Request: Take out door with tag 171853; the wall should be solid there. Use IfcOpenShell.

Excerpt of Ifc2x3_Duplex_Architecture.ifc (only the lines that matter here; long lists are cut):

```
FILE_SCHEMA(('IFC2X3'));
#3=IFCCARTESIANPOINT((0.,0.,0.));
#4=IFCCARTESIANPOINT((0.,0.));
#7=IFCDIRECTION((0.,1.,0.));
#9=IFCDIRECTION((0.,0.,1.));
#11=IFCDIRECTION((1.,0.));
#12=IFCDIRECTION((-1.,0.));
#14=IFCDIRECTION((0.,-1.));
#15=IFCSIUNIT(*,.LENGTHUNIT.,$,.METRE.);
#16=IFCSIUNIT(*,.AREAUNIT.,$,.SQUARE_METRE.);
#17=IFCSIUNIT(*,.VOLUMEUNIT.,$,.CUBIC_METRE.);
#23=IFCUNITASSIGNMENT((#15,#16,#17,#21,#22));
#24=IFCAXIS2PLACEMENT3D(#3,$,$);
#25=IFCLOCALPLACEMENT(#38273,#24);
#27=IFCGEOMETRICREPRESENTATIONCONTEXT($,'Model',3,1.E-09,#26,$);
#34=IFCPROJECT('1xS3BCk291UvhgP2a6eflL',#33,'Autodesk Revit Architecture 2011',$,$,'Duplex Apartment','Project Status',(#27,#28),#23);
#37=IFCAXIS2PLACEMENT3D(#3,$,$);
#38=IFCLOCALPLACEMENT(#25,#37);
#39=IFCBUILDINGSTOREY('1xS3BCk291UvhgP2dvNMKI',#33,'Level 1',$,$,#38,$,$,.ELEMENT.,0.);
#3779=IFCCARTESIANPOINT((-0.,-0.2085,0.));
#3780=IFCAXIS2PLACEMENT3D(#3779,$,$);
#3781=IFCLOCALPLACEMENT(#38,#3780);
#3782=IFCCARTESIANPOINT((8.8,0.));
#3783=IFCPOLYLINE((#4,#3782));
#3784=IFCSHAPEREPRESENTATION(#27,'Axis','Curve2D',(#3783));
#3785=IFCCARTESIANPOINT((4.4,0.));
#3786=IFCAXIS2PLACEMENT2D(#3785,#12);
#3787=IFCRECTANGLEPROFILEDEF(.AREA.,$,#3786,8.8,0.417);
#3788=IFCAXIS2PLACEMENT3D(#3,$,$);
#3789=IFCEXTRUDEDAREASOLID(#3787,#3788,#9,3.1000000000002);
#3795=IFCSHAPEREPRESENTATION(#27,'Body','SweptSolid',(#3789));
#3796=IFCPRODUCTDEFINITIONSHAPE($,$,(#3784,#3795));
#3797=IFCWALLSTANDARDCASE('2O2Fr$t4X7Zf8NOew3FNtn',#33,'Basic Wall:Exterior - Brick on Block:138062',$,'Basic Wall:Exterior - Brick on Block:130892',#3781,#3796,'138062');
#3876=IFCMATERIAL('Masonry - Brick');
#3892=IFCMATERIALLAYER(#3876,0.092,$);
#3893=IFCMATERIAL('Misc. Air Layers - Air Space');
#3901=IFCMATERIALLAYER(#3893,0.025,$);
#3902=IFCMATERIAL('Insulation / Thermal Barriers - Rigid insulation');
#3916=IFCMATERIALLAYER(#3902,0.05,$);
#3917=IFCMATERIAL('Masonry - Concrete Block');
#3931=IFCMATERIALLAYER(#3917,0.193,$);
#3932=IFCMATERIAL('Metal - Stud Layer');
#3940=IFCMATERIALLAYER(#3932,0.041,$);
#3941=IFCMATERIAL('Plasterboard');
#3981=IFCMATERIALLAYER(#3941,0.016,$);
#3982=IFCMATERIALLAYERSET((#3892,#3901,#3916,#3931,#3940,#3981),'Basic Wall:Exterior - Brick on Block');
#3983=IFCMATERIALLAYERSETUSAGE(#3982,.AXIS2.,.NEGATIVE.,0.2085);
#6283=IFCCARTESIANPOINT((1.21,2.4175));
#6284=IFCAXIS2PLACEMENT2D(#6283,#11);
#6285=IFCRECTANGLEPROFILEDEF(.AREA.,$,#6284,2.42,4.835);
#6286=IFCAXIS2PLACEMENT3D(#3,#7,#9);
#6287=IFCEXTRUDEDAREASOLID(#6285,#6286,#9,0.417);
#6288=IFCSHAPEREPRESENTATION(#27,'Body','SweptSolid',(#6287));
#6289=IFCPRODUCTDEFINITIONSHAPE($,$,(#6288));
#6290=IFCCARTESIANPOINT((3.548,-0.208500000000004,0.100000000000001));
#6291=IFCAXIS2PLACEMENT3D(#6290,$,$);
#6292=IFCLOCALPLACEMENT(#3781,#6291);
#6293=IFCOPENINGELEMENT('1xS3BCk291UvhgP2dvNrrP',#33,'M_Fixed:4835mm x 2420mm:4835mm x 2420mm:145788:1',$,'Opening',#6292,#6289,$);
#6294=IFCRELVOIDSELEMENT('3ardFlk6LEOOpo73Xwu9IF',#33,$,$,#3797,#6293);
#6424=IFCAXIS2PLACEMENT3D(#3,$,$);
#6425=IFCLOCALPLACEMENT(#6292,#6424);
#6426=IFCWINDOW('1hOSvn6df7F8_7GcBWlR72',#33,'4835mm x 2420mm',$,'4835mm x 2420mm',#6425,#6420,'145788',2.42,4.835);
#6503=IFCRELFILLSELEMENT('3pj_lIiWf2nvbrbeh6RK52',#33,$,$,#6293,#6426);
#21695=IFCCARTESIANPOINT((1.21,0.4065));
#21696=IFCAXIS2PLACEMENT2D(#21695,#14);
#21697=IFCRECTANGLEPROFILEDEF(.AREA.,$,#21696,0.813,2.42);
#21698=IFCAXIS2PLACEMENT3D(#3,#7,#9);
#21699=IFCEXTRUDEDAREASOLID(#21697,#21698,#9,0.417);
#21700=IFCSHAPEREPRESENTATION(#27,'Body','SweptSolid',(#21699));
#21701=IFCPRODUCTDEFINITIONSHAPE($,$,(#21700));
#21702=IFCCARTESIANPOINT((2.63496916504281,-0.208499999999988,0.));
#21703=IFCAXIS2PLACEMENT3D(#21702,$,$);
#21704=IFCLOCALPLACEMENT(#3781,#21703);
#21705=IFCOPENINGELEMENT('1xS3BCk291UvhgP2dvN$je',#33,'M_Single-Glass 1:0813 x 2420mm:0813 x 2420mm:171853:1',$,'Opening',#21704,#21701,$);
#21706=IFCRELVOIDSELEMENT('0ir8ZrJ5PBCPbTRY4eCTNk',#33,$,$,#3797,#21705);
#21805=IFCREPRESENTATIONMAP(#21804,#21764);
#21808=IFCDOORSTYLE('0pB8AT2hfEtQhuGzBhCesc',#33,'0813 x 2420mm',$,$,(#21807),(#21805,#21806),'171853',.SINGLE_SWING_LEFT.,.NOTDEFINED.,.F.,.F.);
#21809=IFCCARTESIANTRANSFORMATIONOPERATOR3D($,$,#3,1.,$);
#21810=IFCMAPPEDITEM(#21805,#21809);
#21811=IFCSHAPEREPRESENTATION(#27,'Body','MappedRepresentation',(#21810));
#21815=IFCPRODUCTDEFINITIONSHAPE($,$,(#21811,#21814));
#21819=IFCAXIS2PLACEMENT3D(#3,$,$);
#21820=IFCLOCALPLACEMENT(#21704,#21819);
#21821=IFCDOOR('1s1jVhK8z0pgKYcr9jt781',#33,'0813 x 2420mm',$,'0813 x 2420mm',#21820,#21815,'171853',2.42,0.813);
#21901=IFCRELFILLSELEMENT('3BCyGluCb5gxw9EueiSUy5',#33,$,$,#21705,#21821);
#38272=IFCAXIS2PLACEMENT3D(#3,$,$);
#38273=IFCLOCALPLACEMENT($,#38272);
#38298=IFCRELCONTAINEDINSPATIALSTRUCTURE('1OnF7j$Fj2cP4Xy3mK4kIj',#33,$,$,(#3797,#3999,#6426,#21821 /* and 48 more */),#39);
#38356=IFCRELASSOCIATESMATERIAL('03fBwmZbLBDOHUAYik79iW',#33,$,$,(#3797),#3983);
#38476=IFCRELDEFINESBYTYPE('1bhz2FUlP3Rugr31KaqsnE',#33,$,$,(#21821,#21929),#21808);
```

```python
import ifcopenshell
import ifcopenshell.api.feature
import ifcopenshell.api.root
import ifcopenshell.geom
import ifcopenshell.util.shape

model = ifcopenshell.open("Ifc2x3_Duplex_Architecture.ifc")
settings = ifcopenshell.geom.settings()


def volume(element):
    """Net volume in cubic metres, openings subtracted."""
    shape = ifcopenshell.geom.create_shape(settings, element)
    return ifcopenshell.util.shape.get_volume(shape.geometry)


door = model.by_guid("1s1jVhK8z0pgKYcr9jt781")
opening = door.FillsVoids[0].RelatingOpeningElement
wall = opening.VoidsElements[0].RelatingBuildingElement
before = volume(wall)

ifcopenshell.api.root.remove_product(model, product=door)
ifcopenshell.api.feature.remove_feature(model, feature=opening)

after = volume(wall)

print(f"wall volume {before:.3f} -> {after:.3f} m3")

model.write("Ifc2x3_Duplex_Architecture_rev.ifc")
```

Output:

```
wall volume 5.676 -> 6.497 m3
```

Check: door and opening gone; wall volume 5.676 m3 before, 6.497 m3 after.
